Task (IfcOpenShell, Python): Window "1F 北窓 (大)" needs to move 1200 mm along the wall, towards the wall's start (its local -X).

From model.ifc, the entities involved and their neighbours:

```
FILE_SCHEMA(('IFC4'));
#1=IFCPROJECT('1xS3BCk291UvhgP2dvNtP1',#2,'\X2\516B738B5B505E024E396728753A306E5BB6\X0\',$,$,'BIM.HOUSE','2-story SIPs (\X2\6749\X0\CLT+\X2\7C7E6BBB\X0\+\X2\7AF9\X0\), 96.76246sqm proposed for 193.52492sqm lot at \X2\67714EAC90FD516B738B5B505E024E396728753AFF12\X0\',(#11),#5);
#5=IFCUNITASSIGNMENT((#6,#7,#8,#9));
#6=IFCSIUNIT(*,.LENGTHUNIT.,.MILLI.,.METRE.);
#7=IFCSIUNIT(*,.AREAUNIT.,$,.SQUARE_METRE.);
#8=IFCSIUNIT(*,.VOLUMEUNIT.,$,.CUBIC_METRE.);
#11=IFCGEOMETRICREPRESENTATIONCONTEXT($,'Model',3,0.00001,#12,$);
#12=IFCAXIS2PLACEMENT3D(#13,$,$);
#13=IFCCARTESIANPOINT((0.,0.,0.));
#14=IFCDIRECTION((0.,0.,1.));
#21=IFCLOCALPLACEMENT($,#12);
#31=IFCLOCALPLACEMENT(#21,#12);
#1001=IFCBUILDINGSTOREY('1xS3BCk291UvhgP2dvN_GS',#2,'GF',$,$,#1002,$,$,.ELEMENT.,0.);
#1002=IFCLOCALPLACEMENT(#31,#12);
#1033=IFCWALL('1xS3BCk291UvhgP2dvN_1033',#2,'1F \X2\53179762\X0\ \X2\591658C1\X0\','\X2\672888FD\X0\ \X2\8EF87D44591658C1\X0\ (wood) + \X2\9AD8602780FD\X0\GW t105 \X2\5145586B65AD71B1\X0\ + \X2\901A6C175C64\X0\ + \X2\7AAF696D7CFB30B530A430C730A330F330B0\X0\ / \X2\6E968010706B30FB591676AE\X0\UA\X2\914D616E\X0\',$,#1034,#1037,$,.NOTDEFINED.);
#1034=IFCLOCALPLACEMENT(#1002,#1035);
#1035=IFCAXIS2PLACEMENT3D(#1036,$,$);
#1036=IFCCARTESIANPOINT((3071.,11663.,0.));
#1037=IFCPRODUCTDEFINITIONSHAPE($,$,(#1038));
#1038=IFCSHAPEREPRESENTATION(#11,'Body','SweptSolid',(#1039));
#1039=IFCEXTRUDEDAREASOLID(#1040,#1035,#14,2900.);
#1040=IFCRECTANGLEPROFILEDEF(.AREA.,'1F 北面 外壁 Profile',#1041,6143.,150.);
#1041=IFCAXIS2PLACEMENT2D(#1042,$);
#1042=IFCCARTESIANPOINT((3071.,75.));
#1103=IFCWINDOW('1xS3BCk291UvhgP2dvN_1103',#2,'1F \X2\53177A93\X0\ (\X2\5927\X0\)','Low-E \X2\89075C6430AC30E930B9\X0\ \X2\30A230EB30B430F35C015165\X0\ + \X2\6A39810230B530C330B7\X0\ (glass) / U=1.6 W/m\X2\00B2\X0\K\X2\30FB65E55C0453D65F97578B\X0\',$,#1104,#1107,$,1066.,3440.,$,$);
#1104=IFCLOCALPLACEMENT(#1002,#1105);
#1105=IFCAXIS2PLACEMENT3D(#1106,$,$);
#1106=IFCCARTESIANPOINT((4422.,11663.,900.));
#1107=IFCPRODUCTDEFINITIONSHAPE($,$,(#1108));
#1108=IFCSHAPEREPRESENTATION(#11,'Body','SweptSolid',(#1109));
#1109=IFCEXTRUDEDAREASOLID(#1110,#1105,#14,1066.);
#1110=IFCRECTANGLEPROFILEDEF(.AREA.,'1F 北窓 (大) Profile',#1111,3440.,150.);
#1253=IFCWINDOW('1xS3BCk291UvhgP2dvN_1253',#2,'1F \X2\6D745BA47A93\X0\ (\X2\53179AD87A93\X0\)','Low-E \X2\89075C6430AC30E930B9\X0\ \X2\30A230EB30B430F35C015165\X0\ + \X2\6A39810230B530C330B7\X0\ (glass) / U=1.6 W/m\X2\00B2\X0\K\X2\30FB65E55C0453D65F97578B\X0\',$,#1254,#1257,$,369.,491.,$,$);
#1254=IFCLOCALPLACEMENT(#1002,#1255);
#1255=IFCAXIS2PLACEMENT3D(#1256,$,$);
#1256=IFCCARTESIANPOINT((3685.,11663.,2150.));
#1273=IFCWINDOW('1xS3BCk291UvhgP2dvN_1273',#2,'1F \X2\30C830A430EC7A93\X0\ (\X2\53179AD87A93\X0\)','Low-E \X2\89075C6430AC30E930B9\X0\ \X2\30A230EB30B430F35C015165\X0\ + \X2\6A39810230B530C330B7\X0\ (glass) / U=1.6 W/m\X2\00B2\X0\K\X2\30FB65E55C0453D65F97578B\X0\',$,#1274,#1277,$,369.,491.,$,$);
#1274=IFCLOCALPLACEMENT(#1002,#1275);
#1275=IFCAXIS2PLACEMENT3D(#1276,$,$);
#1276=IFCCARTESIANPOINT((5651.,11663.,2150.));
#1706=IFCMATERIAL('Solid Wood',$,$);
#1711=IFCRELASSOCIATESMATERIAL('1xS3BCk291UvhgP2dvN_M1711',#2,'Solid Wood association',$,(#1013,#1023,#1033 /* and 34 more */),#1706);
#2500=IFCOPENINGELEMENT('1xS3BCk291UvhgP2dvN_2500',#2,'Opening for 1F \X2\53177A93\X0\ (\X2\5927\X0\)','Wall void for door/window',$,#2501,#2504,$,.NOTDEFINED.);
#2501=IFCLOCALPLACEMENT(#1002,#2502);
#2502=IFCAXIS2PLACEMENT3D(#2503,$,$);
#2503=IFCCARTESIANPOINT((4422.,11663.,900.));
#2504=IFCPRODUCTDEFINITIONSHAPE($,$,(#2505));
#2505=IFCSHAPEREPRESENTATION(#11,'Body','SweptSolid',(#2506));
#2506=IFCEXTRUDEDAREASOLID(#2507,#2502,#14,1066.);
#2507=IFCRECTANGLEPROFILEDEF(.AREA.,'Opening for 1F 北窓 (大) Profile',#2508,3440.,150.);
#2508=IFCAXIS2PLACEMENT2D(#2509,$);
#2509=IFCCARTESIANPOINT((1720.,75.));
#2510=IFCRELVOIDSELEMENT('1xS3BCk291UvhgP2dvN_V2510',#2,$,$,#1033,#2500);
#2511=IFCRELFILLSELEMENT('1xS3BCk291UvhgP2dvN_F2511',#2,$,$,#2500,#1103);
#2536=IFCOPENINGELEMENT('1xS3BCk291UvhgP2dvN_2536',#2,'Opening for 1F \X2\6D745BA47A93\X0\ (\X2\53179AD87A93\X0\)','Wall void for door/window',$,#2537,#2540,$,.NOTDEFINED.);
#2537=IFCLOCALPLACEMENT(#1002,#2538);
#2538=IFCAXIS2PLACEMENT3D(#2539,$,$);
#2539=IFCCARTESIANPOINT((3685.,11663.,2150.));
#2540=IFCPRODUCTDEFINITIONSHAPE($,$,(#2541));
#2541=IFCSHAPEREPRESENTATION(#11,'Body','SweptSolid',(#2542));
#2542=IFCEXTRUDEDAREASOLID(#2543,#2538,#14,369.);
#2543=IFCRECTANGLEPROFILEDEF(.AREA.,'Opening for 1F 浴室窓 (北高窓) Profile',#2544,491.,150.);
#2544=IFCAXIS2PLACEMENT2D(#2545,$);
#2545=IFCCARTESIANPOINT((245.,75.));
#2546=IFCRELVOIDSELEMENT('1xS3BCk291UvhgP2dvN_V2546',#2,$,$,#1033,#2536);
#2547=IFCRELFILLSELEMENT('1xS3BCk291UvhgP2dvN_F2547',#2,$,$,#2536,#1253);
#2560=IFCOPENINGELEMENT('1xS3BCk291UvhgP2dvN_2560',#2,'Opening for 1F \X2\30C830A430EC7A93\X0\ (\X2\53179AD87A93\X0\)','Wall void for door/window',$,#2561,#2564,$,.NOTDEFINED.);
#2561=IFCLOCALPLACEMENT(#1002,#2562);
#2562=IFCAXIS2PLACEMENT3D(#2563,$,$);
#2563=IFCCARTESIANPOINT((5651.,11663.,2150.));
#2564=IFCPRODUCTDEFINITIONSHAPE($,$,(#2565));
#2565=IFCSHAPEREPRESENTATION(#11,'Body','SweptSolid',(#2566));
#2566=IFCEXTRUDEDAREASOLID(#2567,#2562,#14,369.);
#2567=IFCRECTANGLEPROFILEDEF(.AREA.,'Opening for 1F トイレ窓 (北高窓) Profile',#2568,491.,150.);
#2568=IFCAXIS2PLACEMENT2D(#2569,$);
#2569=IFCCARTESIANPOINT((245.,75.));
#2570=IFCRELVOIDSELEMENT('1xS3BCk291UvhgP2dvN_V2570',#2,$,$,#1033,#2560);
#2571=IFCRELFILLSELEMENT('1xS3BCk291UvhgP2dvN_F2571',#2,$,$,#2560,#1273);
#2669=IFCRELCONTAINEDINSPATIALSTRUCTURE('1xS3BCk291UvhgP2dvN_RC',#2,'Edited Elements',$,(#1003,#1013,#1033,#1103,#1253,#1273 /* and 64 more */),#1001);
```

```python
import ifcopenshell
import ifcopenshell.api.geometry
import ifcopenshell.util.placement
import ifcopenshell.util.unit

model = ifcopenshell.open("model.ifc")
unit_scale = ifcopenshell.util.unit.calculate_unit_scale(model)

window = model.by_guid("1xS3BCk291UvhgP2dvN_1103")
opening = window.FillsVoids[0].RelatingOpeningElement
wall = opening.VoidsElements[0].RelatingBuildingElement

wall_matrix = ifcopenshell.util.placement.get_local_placement(wall.ObjectPlacement)
shift = wall_matrix[:3, 0] * -1.2 / unit_scale
before = ifcopenshell.util.placement.get_local_placement(window.ObjectPlacement)[:3, 3].copy()

# The window is not placed relative to its opening, so move both.
for product in (opening, window):
    matrix = ifcopenshell.util.placement.get_local_placement(product.ObjectPlacement)
    matrix[:3, 3] += shift
    ifcopenshell.api.geometry.edit_object_placement(model, product=product, matrix=matrix, is_si=False)

after = ifcopenshell.util.placement.get_local_placement(window.ObjectPlacement)[:3, 3]
print("window moved by", (after - before).round(3) + 0.0)

model.write("model_rev.ifc")
```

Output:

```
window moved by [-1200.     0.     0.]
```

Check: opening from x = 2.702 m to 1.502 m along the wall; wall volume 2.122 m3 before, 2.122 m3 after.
